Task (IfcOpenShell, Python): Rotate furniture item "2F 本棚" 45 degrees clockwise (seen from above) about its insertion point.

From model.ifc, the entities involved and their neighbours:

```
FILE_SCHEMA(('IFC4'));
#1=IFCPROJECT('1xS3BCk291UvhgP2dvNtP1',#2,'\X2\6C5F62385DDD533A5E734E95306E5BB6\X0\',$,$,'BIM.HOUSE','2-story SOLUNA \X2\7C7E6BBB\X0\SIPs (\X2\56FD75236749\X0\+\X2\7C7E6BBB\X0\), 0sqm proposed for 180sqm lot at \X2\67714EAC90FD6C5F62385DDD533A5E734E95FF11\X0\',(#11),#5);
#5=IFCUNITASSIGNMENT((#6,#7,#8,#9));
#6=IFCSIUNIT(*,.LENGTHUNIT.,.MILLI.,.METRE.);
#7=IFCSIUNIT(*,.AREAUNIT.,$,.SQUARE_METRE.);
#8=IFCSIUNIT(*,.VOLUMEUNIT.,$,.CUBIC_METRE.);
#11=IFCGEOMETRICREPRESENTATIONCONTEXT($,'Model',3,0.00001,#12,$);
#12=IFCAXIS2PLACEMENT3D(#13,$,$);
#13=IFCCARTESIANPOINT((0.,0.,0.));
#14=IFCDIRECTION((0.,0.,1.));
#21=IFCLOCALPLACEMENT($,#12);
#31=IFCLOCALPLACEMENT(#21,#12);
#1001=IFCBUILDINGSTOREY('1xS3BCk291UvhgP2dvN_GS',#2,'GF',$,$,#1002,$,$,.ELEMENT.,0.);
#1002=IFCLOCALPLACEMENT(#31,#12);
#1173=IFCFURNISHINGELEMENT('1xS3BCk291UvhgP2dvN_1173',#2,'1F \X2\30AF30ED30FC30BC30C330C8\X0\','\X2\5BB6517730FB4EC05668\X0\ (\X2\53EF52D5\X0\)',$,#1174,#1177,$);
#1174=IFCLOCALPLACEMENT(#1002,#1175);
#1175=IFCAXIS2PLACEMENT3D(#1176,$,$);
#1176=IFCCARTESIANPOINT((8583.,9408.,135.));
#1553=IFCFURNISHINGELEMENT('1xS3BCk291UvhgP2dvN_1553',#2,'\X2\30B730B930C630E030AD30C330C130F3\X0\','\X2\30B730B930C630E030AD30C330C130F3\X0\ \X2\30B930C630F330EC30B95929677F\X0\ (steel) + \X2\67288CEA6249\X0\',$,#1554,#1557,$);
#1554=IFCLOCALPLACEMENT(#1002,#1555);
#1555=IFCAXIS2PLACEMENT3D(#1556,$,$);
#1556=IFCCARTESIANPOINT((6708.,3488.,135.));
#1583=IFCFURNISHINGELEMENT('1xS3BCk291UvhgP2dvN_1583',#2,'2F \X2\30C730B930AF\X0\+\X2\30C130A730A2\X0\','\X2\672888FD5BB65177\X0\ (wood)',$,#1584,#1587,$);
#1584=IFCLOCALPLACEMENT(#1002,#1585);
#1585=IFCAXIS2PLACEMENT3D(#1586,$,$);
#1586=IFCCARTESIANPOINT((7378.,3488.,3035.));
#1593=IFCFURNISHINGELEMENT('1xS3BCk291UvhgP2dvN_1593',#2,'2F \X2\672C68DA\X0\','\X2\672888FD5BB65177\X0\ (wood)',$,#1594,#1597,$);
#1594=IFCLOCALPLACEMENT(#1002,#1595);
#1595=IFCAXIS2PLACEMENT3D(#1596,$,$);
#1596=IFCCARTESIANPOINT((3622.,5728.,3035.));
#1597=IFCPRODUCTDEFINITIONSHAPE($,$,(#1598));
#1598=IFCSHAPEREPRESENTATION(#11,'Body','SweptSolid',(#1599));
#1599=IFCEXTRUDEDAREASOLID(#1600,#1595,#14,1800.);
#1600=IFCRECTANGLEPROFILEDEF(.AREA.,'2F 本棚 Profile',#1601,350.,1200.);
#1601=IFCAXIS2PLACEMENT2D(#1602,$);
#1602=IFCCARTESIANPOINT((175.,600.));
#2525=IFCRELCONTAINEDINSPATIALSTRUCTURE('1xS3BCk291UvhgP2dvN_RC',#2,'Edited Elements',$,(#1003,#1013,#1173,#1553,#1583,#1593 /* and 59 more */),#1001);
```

```python
import ifcopenshell
import ifcopenshell.api.geometry
import ifcopenshell.util.placement

model = ifcopenshell.open("model.ifc")

item = model.by_id(1593)
matrix = ifcopenshell.util.placement.get_local_placement(item.ObjectPlacement)
matrix = matrix @ ifcopenshell.util.placement.rotation(-45, "Z")
ifcopenshell.api.geometry.edit_object_placement(model, product=item, matrix=matrix, is_si=False)

print(ifcopenshell.util.placement.get_local_placement(item.ObjectPlacement).round(3) + 0.0)

model.write("model-out.ifc")
```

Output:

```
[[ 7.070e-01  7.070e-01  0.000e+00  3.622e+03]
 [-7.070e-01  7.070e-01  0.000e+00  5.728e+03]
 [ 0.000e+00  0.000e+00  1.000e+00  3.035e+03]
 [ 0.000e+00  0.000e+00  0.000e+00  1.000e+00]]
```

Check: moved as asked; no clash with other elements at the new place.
